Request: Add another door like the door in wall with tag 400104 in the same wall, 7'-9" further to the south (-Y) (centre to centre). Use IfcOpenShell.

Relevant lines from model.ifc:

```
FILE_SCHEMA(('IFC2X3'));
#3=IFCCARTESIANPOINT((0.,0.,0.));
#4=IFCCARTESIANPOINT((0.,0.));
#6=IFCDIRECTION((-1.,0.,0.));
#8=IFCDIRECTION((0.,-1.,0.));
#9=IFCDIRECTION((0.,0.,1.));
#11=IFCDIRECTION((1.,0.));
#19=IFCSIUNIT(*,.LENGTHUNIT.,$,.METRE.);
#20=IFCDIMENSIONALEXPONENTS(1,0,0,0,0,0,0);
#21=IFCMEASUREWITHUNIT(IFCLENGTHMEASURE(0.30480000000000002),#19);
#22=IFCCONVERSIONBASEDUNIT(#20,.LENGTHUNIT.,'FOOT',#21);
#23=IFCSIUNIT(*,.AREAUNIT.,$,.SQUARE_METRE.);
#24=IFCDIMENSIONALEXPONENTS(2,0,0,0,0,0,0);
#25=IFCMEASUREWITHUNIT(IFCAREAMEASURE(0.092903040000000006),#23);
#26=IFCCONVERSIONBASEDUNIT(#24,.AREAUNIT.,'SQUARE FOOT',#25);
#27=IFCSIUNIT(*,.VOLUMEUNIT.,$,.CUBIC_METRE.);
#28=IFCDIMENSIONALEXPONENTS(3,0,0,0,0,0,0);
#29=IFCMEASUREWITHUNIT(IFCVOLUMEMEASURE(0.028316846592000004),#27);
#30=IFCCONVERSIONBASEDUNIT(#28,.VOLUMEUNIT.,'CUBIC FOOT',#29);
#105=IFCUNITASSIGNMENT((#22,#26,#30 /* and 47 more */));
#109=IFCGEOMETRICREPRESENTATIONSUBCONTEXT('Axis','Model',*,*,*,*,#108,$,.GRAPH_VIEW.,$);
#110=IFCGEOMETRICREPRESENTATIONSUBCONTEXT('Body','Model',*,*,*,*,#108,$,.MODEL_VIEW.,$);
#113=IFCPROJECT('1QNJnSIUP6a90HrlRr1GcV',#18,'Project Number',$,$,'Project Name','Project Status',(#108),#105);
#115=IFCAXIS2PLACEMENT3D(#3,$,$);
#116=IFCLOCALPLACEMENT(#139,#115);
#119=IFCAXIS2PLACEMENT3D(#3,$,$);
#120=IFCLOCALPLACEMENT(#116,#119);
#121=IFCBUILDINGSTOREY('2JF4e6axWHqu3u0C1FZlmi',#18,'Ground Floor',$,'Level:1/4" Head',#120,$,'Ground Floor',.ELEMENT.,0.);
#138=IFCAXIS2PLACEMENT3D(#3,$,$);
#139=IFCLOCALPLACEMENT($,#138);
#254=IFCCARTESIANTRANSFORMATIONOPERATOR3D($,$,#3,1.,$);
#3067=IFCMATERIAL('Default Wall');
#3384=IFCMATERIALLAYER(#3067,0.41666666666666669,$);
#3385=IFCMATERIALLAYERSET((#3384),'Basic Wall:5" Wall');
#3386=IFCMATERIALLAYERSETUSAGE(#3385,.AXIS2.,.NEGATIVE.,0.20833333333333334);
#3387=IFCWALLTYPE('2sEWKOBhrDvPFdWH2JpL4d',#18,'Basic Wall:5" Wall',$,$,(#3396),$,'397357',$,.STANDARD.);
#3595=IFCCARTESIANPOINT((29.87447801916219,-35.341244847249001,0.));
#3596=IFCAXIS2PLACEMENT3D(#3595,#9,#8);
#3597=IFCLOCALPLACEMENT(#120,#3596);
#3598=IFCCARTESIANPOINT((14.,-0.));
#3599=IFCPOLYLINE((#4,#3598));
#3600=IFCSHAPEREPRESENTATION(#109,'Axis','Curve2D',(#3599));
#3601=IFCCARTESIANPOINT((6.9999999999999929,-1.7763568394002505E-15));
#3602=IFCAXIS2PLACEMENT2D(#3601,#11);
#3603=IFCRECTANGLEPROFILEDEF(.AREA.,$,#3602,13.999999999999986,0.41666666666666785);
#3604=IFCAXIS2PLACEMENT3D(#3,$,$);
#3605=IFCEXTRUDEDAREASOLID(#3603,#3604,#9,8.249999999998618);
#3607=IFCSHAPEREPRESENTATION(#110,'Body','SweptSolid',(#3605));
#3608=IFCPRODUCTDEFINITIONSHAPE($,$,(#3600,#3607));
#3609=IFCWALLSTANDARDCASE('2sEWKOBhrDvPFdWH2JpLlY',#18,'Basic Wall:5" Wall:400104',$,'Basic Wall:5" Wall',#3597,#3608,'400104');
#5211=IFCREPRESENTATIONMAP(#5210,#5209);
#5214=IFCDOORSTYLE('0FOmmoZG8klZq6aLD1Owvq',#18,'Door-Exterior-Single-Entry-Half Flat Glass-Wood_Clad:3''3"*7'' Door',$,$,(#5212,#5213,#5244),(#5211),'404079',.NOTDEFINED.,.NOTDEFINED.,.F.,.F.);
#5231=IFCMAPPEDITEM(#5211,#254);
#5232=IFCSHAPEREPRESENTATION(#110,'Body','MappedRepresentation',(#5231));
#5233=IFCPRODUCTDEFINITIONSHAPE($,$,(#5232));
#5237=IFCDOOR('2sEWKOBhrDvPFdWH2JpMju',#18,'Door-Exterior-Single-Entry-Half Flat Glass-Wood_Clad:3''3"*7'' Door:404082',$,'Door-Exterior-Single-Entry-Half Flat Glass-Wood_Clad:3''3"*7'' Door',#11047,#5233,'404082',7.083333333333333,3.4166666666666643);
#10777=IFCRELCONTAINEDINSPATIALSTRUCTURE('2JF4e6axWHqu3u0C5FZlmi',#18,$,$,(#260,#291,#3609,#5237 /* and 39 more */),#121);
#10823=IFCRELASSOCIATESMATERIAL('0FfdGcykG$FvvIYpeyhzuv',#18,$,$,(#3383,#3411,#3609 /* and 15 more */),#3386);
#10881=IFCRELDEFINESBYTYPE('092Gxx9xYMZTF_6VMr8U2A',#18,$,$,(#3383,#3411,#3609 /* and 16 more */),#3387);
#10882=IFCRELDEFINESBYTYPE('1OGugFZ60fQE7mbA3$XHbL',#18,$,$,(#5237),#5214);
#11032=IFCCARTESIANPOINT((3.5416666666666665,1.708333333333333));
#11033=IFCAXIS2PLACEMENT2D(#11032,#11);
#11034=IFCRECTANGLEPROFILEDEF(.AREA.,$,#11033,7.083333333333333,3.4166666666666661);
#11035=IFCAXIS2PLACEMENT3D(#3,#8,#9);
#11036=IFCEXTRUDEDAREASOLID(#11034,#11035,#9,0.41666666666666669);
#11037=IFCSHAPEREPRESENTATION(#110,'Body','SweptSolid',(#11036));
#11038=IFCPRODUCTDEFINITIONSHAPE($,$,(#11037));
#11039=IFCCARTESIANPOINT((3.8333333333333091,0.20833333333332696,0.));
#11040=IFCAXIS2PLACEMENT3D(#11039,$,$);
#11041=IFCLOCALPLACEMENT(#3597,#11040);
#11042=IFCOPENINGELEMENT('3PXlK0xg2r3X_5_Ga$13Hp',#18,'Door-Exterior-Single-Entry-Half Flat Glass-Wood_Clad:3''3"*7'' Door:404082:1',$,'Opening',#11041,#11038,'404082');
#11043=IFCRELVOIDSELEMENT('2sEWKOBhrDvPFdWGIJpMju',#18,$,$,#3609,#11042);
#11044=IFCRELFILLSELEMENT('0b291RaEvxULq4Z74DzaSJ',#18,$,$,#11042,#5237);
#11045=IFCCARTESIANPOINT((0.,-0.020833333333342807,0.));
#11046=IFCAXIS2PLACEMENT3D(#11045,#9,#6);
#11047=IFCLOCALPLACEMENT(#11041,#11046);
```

```python
import ifcopenshell
import ifcopenshell.api.feature
import ifcopenshell.api.geometry
import ifcopenshell.api.root
import ifcopenshell.geom
import ifcopenshell.util.element
import ifcopenshell.util.placement
import ifcopenshell.util.shape
import ifcopenshell.util.unit

model = ifcopenshell.open("model.ifc")
unit_scale = ifcopenshell.util.unit.calculate_unit_scale(model)
settings = ifcopenshell.geom.settings()


def volume(element):
    """Net volume in cubic metres, openings subtracted."""
    shape = ifcopenshell.geom.create_shape(settings, element)
    return ifcopenshell.util.shape.get_volume(shape.geometry)


def reuse_history(source, copy):
    """copy_class also copies each property set's owner history, people and application; keep the originals."""
    for rel in copy.IsDefinedBy:
        if rel.is_a("IfcRelDefinesByProperties") and (history := rel.RelatingPropertyDefinition.OwnerHistory):
            rel.RelatingPropertyDefinition.OwnerHistory = source.OwnerHistory
            ifcopenshell.util.element.remove_deep2(model, history)


door = model.by_guid("2sEWKOBhrDvPFdWH2JpMju")
opening = door.FillsVoids[0].RelatingOpeningElement
wall = opening.VoidsElements[0].RelatingBuildingElement
before = volume(wall)
shift = ifcopenshell.util.placement.get_local_placement(wall.ObjectPlacement)[:3, 0] * 93 * 0.0254 / unit_scale

# copy_class copies the void relationship, type, container and properties, but no geometry.
new_opening = ifcopenshell.api.root.copy_class(model, product=opening)
new_opening.Representation = ifcopenshell.util.element.copy_deep(
    model, opening.Representation, exclude=["IfcGeometricRepresentationContext", "IfcRepresentationMap"]
)
new_opening.Name = 'Door-Exterior-Single-Entry-Half Flat Glass-Wood_Clad:3\'3"*7\' Door'
new_opening.Tag = None
new_door = ifcopenshell.api.root.copy_class(model, product=door)
new_door.Representation = ifcopenshell.util.element.copy_deep(
    model, door.Representation, exclude=["IfcGeometricRepresentationContext", "IfcRepresentationMap"]
)
new_door.Name = 'Door-Exterior-Single-Entry-Half Flat Glass-Wood_Clad:3\'3"*7\' Door'
new_door.Tag = None
reuse_history(door, new_door)
fills = ifcopenshell.api.feature.add_filling(model, opening=new_opening, element=new_door)
fills.OwnerHistory = new_door.OwnerHistory  # required in IFC2X3

for old, new in ((opening, new_opening), (door, new_door)):
    matrix = ifcopenshell.util.placement.get_local_placement(old.ObjectPlacement)
    matrix[:3, 3] += shift
    ifcopenshell.api.geometry.edit_object_placement(model, product=new, matrix=matrix, is_si=False)

after = volume(wall)

print(f"wall volume {before:.3f} -> {after:.3f} m3")

model.write("model_edited.ifc")
```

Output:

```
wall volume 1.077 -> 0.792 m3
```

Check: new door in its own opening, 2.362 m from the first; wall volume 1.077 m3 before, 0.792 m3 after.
